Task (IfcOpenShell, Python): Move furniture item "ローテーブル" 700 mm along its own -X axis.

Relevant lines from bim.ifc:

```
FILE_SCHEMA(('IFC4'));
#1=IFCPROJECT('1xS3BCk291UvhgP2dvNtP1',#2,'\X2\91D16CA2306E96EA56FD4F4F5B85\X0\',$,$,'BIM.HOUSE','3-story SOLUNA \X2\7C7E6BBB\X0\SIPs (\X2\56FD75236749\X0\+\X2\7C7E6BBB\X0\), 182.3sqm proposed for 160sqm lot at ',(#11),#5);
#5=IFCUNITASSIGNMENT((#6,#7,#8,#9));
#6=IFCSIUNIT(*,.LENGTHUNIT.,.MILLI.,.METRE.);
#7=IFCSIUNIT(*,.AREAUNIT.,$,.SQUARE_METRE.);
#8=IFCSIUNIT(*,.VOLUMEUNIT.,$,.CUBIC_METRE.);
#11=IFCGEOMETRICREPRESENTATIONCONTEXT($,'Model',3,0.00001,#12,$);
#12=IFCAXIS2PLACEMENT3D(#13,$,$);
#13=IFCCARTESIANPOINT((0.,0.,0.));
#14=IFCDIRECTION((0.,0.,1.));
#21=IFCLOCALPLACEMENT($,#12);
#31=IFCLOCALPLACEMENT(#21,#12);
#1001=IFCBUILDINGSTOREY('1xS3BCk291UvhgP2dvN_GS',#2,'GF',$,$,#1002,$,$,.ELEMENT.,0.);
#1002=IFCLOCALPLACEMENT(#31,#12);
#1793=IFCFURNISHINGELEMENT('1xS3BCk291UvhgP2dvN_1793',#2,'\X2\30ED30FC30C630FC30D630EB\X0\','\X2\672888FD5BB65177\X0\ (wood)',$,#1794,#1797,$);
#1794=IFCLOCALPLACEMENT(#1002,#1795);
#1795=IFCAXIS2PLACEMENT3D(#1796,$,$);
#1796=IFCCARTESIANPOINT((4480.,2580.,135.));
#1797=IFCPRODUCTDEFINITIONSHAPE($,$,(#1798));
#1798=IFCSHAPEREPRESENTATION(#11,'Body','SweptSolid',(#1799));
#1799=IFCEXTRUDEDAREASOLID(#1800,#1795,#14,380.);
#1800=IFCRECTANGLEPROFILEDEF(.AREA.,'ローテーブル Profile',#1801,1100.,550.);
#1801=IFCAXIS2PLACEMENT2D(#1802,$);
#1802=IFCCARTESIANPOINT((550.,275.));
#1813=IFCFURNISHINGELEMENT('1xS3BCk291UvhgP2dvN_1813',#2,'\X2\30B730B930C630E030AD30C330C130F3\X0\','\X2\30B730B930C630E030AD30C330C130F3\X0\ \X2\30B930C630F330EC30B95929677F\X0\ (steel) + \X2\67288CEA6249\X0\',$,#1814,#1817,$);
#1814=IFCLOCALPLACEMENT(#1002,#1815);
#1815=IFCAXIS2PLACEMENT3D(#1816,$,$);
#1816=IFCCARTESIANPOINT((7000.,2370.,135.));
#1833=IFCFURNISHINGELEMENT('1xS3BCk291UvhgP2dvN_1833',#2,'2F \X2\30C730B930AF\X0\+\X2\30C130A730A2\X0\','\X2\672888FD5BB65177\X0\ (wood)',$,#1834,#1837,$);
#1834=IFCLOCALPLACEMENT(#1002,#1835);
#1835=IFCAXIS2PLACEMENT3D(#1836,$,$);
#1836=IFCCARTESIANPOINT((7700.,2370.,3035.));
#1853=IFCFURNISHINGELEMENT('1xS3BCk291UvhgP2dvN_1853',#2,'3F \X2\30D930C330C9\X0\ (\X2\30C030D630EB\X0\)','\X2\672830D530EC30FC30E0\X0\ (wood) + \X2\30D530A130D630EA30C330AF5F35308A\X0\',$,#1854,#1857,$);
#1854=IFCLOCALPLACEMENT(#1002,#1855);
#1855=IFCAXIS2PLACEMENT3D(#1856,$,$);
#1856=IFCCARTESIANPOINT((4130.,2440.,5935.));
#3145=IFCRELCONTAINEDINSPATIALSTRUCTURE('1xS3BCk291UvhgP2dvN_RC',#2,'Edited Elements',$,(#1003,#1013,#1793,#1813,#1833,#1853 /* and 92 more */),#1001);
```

```python
import ifcopenshell
import ifcopenshell.api.geometry
import ifcopenshell.util.placement

model = ifcopenshell.open("bim.ifc")

item = model.by_guid("1xS3BCk291UvhgP2dvN_1793")
matrix = ifcopenshell.util.placement.get_local_placement(item.ObjectPlacement)
matrix[:3, 3] -= matrix[:3, 0] * 700.0
ifcopenshell.api.geometry.edit_object_placement(model, product=item, matrix=matrix, is_si=False)

print(ifcopenshell.util.placement.get_local_placement(item.ObjectPlacement).round(3) + 0.0)

model.write("bim_v2.ifc")
```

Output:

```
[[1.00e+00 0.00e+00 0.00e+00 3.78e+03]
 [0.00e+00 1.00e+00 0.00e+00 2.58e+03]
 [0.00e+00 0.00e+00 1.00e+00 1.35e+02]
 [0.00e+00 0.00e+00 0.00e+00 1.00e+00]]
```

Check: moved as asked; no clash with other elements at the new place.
